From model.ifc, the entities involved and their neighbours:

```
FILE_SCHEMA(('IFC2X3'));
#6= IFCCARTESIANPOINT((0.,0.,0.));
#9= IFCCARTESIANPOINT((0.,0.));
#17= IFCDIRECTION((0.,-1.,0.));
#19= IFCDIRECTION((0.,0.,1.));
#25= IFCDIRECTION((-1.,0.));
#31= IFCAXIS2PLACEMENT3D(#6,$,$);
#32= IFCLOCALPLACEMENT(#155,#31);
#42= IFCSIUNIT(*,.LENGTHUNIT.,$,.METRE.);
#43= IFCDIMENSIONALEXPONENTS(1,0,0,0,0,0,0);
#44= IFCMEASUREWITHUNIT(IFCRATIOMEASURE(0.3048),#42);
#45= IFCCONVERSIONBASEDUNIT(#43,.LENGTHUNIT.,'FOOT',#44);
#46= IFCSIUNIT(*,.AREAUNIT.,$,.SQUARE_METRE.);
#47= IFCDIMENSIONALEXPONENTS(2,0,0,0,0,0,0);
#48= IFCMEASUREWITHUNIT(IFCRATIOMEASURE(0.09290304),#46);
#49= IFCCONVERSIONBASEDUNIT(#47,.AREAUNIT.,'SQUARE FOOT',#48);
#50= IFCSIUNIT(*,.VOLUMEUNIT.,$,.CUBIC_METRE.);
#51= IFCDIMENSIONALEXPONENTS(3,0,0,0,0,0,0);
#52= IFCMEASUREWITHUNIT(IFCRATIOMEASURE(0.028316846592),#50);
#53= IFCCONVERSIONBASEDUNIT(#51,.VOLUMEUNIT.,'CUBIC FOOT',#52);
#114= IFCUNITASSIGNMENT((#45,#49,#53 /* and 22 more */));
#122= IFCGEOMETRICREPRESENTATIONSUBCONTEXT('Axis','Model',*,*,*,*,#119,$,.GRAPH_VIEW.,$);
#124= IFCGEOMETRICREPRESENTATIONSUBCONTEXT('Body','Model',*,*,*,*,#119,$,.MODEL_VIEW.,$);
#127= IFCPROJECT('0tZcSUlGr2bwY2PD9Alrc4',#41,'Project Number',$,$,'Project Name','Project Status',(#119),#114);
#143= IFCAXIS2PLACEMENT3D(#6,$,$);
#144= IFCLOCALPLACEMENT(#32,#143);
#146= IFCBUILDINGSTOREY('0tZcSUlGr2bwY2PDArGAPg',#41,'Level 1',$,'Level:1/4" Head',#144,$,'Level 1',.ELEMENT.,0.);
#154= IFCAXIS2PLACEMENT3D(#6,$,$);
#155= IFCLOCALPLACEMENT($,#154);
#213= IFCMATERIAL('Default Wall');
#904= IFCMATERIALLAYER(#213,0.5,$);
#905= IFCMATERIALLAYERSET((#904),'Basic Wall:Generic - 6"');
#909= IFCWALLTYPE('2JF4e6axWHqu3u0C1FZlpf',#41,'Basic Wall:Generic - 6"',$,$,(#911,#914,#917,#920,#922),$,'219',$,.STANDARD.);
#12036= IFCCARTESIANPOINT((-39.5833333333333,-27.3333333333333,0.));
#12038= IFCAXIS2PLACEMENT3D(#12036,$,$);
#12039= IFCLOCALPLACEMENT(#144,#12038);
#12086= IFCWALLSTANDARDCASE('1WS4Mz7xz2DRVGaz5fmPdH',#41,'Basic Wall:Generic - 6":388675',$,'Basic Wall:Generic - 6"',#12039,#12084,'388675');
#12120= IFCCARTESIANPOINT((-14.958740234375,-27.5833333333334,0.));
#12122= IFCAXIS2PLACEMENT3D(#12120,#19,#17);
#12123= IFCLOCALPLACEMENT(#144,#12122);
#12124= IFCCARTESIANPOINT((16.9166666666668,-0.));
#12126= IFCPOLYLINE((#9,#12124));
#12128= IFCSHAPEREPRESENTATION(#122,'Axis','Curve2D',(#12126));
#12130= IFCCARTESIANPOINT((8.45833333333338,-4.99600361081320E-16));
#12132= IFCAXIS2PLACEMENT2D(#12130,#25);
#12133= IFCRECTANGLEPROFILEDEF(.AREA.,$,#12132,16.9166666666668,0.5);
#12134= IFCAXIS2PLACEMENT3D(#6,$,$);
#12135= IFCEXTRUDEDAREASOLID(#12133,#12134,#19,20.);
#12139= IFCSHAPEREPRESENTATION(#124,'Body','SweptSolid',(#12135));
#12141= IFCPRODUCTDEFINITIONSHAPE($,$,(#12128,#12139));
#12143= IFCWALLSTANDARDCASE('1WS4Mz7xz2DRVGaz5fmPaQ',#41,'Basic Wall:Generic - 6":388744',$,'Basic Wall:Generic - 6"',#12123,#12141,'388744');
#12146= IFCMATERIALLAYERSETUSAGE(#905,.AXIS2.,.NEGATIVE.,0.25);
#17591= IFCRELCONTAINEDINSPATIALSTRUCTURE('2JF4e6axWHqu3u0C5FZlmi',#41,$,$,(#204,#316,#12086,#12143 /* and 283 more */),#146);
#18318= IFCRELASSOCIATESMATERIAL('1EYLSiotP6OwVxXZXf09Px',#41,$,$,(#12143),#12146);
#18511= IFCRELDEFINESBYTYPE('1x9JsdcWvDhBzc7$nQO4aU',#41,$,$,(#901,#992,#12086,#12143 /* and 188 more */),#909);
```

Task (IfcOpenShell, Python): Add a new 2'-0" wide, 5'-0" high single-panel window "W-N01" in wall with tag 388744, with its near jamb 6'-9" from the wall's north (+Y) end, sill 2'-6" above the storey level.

```python
import numpy as np
import ifcopenshell
import ifcopenshell.api.feature
import ifcopenshell.api.geometry
import ifcopenshell.api.root
import ifcopenshell.api.spatial
import ifcopenshell.api.type
import ifcopenshell.geom
import ifcopenshell.util.element
import ifcopenshell.util.placement
import ifcopenshell.util.representation
import ifcopenshell.util.shape
import ifcopenshell.util.unit

model = ifcopenshell.open("model.ifc")
unit_scale = ifcopenshell.util.unit.calculate_unit_scale(model)
settings = ifcopenshell.geom.settings()


def volume(element):
    """Net volume in cubic metres, openings subtracted."""
    shape = ifcopenshell.geom.create_shape(settings, element)
    return ifcopenshell.util.shape.get_volume(shape.geometry)


wall = model.by_guid("1WS4Mz7xz2DRVGaz5fmPaQ")
storey = ifcopenshell.util.element.get_container(wall, ifc_class="IfcBuildingStorey")
context = ifcopenshell.util.representation.get_context(model, "Model", "Body", "MODEL_VIEW")
before = volume(wall)

width, height, from_end, sill = 0.6096, 1.524, 2.0574, 0.762  # metres

# The wall runs along its own X axis, and the end named is its -X end.
wall_shape = ifcopenshell.geom.create_shape(settings, wall)
x, y, z = ifcopenshell.util.shape.get_vertices(wall_shape.geometry).T
start = x.min() + from_end
face, thickness = float(y.min()), float(y.max() - y.min())
wall_matrix = ifcopenshell.util.placement.get_local_placement(wall.ObjectPlacement)
level = ifcopenshell.util.placement.get_local_placement(storey.ObjectPlacement)[2, 3]


def in_wall(x, y):
    """Placement at x, y metres in the wall's axes, at sill height."""
    matrix = wall_matrix.copy()
    matrix[:, 3] = wall_matrix @ np.array([x / unit_scale, y / unit_scale, 0.0, 1.0])
    matrix[2, 3] = level + sill / unit_scale
    return matrix


# Opening: a box that overshoots both wall faces by 50 mm.
opening = ifcopenshell.api.root.create_entity(model, ifc_class="IfcOpeningElement")
box = ifcopenshell.api.geometry.add_wall_representation(
    model, context=context, length=width, height=height, thickness=thickness + 0.1
)
ifcopenshell.api.geometry.assign_representation(model, product=opening, representation=box)
ifcopenshell.api.geometry.edit_object_placement(model, product=opening, matrix=in_wall(start, face - 0.05), is_si=False)
ifcopenshell.api.feature.add_feature(model, feature=opening, element=wall)

window = ifcopenshell.api.root.create_entity(model, ifc_class="IfcWindow", name="W-N01")
window.OverallWidth, window.OverallHeight = width / unit_scale, height / unit_scale
body = ifcopenshell.api.geometry.add_window_representation(
    model,
    context=context,
    overall_width=window.OverallWidth,
    overall_height=window.OverallHeight,
    partition_type="SINGLE_PANEL",
)
ifcopenshell.api.geometry.assign_representation(model, product=window, representation=body)
ifcopenshell.api.spatial.assign_container(model, products=[window], relating_structure=storey)
fills = ifcopenshell.api.feature.add_filling(model, opening=opening, element=window)
fills.OwnerHistory = window.OwnerHistory  # required in IFC2X3

# IFC2X3 keeps the operation on the window style.
style = ifcopenshell.api.root.create_entity(model, ifc_class="IfcWindowStyle", name="W-N01")
style.OperationType, style.ConstructionType = "SINGLE_PANEL", "NOTDEFINED"
style.ParameterTakesPrecedence = style.Sizeable = False
ifcopenshell.api.type.assign_type(model, related_objects=[window], relating_type=style)

# Centre the window in the wall's thickness.
ifcopenshell.api.geometry.edit_object_placement(model, product=window, matrix=in_wall(start, face), is_si=False)
window_shape = ifcopenshell.geom.create_shape(settings, window)
depth = ifcopenshell.util.shape.get_vertices(window_shape.geometry)[:, 1]
offset = face + thickness / 2 - (depth.min() + depth.max()) / 2
ifcopenshell.api.geometry.edit_object_placement(model, product=window, matrix=in_wall(start, offset), is_si=False)

after = volume(wall)

print(f"wall volume {before:.3f} -> {after:.3f} m3")

model.write("model_updated.ifc")
```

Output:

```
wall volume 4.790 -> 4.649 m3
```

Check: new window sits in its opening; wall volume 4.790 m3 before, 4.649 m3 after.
